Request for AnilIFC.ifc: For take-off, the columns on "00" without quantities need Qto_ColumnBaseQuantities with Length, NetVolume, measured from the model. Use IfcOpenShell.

First a look at what the model holds.

```python
import ifcopenshell
import ifcopenshell.util.element
import ifcopenshell.util.unit

model = ifcopenshell.open("AnilIFC.ifc")
print(model.schema)
for unit_type in ("LENGTHUNIT", "AREAUNIT", "VOLUMEUNIT"):
    print(unit_type, ifcopenshell.util.unit.calculate_unit_scale(model, unit_type))
storey = next(s for s in model.by_type("IfcBuildingStorey") if s.Name == "00")
columns = [e for e in ifcopenshell.util.element.get_decomposition(storey) if e.is_a("IfcColumn")]
for e in sorted(columns, key=lambda e: e.id()):
    print(e.id(), e.is_a(), e.Name, list(ifcopenshell.util.element.get_psets(e, qtos_only=True)), sep=" | ")
```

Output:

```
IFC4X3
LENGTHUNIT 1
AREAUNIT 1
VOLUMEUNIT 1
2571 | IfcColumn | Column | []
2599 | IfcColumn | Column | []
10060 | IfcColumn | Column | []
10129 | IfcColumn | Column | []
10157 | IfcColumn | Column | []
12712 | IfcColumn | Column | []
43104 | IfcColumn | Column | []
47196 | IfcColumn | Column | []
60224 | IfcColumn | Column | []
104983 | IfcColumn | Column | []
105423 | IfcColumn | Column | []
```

```python
import ifcopenshell
import ifcopenshell.api.pset
import ifcopenshell.geom
import ifcopenshell.util.element
import ifcopenshell.util.shape
import ifcopenshell.util.unit

model = ifcopenshell.open("AnilIFC.ifc")
unit_scale = ifcopenshell.util.unit.calculate_unit_scale(model)
volume_scale = ifcopenshell.util.unit.calculate_unit_scale(model, "VOLUMEUNIT")
settings = ifcopenshell.geom.settings()

storey = next(s for s in model.by_type("IfcBuildingStorey") if s.Name == "00")
columns = [e for e in ifcopenshell.util.element.get_decomposition(storey) if e.is_a("IfcColumn")]

for e in sorted(columns, key=lambda e: e.id()):
    if ifcopenshell.util.element.get_psets(e, qtos_only=True, should_inherit=False):
        continue
    # Geometry comes back in metres, in the element's own axes.
    shape = ifcopenshell.geom.create_shape(settings, e)
    values = {
        "Length": ifcopenshell.util.shape.get_z(shape.geometry) / unit_scale,
        "NetVolume": ifcopenshell.util.shape.get_volume(shape.geometry) / volume_scale,
    }
    qto = ifcopenshell.api.pset.add_qto(model, product=e, name="Qto_ColumnBaseQuantities")
    ifcopenshell.api.pset.edit_qto(model, qto=qto, properties=values)
    print(e.id(), {k: round(v, 3) for k, v in values.items()})

model.write("AnilIFC_v2.ifc")
```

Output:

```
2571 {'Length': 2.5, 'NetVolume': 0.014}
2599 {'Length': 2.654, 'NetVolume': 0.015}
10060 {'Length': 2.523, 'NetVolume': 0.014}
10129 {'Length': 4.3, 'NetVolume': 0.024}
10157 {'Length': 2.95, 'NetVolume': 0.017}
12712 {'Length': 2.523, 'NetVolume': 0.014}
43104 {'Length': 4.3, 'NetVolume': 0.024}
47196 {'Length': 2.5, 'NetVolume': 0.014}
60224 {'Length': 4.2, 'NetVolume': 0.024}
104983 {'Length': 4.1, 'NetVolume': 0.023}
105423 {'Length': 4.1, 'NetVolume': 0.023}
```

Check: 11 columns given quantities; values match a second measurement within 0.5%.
